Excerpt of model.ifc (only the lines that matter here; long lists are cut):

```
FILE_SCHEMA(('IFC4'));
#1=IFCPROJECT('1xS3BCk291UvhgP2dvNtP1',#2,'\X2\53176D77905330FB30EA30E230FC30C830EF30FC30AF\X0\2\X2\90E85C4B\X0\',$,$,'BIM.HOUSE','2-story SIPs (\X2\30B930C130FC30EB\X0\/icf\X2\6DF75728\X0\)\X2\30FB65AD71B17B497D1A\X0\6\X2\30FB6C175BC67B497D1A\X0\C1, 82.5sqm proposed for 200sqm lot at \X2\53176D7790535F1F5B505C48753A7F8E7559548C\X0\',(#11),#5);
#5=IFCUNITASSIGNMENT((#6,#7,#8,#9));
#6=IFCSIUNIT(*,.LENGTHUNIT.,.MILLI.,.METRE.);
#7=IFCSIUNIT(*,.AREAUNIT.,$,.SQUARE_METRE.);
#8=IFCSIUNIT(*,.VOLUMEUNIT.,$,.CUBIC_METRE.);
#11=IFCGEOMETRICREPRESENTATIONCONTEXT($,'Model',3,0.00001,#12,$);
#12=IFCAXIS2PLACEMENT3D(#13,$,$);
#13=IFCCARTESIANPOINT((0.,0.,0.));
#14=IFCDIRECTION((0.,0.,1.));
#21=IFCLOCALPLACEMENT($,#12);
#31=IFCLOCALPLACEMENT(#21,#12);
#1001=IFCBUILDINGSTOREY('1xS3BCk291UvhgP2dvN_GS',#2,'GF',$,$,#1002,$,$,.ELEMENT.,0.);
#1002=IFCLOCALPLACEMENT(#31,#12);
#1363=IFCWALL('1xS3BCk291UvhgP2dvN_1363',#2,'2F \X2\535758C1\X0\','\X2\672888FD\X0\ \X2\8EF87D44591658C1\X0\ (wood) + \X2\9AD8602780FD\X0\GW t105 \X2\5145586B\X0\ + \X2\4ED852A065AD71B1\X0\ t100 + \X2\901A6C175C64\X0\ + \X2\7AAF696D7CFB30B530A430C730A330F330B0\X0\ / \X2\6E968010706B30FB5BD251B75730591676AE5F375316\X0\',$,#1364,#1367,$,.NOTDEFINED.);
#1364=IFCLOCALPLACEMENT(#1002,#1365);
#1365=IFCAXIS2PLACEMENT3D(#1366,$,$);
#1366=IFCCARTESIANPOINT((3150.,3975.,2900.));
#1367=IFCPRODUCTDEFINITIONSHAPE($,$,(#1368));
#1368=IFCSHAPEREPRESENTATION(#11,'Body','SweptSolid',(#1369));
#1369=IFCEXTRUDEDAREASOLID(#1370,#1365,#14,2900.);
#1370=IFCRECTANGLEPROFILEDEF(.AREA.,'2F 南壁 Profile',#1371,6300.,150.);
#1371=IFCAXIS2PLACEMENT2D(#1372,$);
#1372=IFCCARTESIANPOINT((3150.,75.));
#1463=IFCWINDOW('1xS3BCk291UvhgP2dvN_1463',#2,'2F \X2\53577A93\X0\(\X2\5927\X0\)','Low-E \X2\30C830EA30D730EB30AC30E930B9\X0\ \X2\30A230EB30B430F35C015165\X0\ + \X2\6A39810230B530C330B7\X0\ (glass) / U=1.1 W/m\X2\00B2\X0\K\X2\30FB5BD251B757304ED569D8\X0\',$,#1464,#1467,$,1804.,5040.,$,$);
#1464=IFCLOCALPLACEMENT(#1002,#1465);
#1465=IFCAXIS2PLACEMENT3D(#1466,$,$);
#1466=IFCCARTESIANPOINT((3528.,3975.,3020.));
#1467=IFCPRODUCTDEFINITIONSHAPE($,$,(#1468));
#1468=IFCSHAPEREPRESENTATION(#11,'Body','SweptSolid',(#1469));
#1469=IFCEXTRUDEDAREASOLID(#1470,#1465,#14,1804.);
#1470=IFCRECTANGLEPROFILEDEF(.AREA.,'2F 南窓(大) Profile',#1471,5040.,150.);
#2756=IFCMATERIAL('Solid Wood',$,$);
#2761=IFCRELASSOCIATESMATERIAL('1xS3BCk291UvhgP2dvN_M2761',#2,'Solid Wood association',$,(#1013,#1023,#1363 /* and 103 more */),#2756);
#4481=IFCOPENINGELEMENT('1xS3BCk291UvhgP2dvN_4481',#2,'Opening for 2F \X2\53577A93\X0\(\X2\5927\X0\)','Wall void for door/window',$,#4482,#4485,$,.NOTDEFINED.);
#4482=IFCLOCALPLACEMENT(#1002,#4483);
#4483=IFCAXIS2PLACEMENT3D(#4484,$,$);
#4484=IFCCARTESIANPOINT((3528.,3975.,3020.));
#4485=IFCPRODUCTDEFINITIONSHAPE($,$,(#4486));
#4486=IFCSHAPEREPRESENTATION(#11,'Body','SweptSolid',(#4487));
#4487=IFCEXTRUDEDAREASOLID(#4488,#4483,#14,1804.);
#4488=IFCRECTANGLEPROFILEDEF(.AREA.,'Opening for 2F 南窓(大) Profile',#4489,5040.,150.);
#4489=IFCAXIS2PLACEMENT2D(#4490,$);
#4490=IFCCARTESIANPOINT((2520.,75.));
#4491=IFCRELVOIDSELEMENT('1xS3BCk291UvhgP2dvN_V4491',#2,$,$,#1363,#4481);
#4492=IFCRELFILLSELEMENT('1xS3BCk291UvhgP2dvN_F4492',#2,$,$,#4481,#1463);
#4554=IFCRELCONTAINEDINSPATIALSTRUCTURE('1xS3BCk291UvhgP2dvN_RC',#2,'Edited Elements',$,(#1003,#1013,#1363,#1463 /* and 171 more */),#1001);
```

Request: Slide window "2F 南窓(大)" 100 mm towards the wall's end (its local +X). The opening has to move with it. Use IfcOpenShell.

```python
import ifcopenshell
import ifcopenshell.api.geometry
import ifcopenshell.util.placement

model = ifcopenshell.open("model.ifc")

window = model.by_id(1463)
opening = window.FillsVoids[0].RelatingOpeningElement
wall = opening.VoidsElements[0].RelatingBuildingElement

wall_matrix = ifcopenshell.util.placement.get_local_placement(wall.ObjectPlacement)
shift = wall_matrix[:3, 0] * 100.0
before = ifcopenshell.util.placement.get_local_placement(window.ObjectPlacement)[:3, 3].copy()

# The window is not placed relative to its opening, so move both.
for product in (opening, window):
    matrix = ifcopenshell.util.placement.get_local_placement(product.ObjectPlacement)
    matrix[:3, 3] += shift
    ifcopenshell.api.geometry.edit_object_placement(model, product=product, matrix=matrix, is_si=False)

after = ifcopenshell.util.placement.get_local_placement(window.ObjectPlacement)[:3, 3]
print("window moved by", (after - before).round(3) + 0.0)

model.write("model_edited.ifc")
```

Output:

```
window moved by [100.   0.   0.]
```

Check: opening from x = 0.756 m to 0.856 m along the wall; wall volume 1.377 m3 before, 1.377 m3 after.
